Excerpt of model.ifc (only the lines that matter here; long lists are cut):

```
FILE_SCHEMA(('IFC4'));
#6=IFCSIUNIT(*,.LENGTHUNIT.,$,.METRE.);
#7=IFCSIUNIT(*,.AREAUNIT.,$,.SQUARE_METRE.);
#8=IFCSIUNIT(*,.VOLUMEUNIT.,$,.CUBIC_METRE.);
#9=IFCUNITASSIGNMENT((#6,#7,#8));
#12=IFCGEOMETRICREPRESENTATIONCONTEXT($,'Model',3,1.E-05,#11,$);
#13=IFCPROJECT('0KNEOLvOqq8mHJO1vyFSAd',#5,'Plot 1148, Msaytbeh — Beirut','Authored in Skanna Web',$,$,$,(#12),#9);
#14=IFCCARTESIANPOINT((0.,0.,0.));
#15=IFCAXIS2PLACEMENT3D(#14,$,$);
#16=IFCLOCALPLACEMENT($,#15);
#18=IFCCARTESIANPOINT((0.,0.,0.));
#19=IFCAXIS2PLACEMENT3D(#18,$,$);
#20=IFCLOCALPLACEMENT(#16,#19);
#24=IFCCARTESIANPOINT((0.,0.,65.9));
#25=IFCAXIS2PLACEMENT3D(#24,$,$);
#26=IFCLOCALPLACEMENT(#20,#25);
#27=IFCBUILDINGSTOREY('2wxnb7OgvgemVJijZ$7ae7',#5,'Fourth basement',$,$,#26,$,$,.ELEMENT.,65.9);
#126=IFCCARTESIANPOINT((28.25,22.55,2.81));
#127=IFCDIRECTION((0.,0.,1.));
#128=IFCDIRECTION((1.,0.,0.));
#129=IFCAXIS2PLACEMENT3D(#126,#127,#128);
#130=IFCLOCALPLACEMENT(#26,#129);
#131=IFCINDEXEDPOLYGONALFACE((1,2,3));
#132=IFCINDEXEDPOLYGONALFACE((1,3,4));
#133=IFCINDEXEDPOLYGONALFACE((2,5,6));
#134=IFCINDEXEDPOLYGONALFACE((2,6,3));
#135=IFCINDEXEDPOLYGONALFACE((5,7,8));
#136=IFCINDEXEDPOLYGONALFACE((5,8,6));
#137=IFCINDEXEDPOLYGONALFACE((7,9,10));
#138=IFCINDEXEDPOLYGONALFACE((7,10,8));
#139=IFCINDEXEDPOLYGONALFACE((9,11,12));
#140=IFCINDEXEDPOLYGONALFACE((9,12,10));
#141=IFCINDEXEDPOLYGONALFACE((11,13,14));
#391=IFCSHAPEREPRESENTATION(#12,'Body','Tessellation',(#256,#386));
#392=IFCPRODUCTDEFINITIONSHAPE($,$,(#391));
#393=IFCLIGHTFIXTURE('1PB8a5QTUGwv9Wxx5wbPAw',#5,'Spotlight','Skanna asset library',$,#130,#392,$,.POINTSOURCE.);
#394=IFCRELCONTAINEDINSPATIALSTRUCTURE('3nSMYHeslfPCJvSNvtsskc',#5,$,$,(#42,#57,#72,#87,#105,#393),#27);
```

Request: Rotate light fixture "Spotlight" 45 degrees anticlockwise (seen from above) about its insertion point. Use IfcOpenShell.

```python
import ifcopenshell
import ifcopenshell.api.geometry
import ifcopenshell.util.placement

model = ifcopenshell.open("model.ifc")

item = model.by_guid("1PB8a5QTUGwv9Wxx5wbPAw")
matrix = ifcopenshell.util.placement.get_local_placement(item.ObjectPlacement)
matrix = matrix @ ifcopenshell.util.placement.rotation(45, "Z")
ifcopenshell.api.geometry.edit_object_placement(model, product=item, matrix=matrix, is_si=False)

print(ifcopenshell.util.placement.get_local_placement(item.ObjectPlacement).round(3) + 0.0)

model.write("model_edited.ifc")
```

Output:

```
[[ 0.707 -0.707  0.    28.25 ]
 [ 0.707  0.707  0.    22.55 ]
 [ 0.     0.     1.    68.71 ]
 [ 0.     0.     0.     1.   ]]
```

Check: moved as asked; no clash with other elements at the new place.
